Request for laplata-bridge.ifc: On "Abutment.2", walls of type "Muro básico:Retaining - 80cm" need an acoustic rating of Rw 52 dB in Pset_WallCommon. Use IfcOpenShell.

First a look at what the model holds.

```python
import ifcopenshell
import ifcopenshell.util.element

model = ifcopenshell.open("laplata-bridge.ifc")
print(model.schema)
storey = next(s for s in model.by_type("IfcBuildingStorey") if s.Name == "Abutment.2")
walls = [e for e in ifcopenshell.util.element.get_decomposition(storey) if e.is_a("IfcWall")]
seen = {}
for e in walls:
    element_type = ifcopenshell.util.element.get_type(e)
    key = (element_type.Name if element_type != e and element_type else None, ifcopenshell.util.element.get_pset(e, "Pset_WallCommon", "AcousticRating"))
    seen[key] = seen.get(key, 0) + 1
for (name, value), count in sorted(seen.items(), key=str):
    print(count, "x", name, "|", value)
```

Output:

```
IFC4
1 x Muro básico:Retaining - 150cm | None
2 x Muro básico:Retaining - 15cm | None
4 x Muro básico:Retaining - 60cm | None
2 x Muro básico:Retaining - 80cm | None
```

```python
import ifcopenshell
import ifcopenshell.api.pset
import ifcopenshell.util.element

model = ifcopenshell.open("laplata-bridge.ifc")

storey = next(s for s in model.by_type("IfcBuildingStorey") if s.Name == "Abutment.2")
walls = [e for e in ifcopenshell.util.element.get_decomposition(storey) if e.is_a("IfcWall")]

count = 0
for e in walls:
    element_type = ifcopenshell.util.element.get_type(e)
    if element_type in (None, e) or element_type.Name != "Muro básico:Retaining - 80cm":
        continue
    # add_pset returns the element's existing set when there is one.
    pset = ifcopenshell.api.pset.add_pset(model, product=e, name="Pset_WallCommon")
    ifcopenshell.api.pset.edit_pset(model, pset=pset, properties={"AcousticRating": "Rw 52 dB"})
    count += 1

print(count, "walls updated")

model.write("laplata-bridge_v2.ifc")
```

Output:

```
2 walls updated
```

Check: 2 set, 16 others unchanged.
